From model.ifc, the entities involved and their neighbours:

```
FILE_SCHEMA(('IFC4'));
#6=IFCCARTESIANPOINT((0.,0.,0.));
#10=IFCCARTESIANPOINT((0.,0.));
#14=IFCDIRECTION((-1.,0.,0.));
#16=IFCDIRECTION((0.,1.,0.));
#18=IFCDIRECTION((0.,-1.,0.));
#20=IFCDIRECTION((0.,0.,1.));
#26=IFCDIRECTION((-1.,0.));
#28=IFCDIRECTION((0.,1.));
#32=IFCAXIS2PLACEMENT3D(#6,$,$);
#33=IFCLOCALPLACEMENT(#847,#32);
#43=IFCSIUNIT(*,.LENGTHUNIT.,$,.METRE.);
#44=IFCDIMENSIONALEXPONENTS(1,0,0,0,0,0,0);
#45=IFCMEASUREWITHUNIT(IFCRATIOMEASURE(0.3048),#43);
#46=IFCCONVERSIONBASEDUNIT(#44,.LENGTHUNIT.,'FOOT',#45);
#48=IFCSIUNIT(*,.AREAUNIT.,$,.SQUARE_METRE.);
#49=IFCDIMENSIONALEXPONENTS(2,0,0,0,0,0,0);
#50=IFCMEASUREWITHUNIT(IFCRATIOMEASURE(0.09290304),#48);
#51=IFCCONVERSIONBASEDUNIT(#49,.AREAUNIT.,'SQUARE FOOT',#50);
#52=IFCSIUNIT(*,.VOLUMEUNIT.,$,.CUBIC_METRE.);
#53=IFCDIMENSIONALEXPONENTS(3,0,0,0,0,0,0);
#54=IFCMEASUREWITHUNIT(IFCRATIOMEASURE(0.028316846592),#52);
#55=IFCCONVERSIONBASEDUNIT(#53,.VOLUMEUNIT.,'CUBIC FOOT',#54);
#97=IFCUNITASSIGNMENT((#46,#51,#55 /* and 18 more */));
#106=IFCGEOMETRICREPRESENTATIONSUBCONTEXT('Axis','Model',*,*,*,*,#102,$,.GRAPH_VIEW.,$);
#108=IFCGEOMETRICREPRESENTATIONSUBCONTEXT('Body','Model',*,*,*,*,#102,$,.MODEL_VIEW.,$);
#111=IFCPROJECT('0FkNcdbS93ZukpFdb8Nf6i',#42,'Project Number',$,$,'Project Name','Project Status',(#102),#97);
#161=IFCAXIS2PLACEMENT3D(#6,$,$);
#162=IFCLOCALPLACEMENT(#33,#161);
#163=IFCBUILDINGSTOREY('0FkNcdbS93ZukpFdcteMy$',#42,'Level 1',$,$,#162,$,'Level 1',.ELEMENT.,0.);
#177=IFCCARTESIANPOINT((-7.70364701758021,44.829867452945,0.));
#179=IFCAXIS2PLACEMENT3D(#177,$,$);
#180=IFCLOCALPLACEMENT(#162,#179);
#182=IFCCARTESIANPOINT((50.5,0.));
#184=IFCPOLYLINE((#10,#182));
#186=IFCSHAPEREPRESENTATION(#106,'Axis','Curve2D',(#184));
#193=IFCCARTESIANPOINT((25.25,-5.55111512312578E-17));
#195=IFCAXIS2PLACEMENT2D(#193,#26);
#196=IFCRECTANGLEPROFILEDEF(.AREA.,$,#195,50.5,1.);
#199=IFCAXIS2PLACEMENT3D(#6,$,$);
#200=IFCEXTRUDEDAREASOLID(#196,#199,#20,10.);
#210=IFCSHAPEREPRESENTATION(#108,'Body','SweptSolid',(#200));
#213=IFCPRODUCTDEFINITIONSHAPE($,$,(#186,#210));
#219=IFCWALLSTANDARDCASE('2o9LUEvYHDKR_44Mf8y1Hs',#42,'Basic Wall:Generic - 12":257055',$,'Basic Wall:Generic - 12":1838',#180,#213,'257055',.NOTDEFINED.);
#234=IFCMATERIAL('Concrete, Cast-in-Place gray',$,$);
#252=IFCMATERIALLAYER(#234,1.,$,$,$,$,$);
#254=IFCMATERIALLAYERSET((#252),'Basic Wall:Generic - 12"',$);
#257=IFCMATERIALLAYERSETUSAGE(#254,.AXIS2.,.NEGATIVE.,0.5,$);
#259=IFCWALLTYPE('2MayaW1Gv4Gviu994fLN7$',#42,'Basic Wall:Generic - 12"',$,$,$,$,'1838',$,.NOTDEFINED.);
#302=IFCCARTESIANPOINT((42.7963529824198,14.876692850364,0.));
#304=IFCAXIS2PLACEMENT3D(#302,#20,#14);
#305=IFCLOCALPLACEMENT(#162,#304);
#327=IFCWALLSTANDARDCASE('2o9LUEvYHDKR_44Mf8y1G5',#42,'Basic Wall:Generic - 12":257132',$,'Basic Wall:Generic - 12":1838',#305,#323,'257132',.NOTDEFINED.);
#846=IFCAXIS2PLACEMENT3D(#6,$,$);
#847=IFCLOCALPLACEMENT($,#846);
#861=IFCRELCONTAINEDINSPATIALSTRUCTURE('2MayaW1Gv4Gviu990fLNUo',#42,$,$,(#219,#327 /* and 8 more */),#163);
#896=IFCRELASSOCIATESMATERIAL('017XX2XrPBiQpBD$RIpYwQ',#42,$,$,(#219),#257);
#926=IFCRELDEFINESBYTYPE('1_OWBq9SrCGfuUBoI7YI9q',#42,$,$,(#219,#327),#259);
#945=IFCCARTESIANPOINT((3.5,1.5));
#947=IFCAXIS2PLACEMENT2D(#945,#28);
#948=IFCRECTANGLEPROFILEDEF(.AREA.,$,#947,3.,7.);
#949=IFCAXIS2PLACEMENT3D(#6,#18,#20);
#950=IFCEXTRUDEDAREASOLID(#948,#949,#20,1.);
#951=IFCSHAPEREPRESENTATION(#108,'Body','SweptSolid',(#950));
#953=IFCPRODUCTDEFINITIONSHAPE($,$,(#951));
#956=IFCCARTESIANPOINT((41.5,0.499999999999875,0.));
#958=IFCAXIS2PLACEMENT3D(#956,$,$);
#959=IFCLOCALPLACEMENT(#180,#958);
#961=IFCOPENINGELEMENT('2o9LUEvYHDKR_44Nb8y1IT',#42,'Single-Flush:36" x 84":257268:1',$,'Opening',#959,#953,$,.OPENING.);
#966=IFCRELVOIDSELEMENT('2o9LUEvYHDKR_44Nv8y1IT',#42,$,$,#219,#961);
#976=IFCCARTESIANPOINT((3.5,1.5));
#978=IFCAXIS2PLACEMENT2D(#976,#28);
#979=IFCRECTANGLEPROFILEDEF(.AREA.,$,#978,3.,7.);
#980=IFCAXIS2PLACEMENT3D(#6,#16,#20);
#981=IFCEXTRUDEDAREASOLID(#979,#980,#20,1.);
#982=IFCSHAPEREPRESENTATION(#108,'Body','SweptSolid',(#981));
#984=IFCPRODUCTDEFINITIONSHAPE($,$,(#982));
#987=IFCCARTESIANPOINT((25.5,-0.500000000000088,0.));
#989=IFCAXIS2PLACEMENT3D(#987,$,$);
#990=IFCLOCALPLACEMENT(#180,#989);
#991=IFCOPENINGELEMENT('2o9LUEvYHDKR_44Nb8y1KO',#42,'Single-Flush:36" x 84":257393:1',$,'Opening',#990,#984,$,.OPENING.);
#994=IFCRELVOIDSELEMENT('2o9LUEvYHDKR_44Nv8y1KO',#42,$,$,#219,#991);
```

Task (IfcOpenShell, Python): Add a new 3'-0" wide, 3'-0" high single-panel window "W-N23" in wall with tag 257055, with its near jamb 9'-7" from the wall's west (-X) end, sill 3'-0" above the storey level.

```python
import numpy as np
import ifcopenshell
import ifcopenshell.api.feature
import ifcopenshell.api.geometry
import ifcopenshell.api.root
import ifcopenshell.api.spatial
import ifcopenshell.geom
import ifcopenshell.util.element
import ifcopenshell.util.placement
import ifcopenshell.util.representation
import ifcopenshell.util.shape
import ifcopenshell.util.unit

model = ifcopenshell.open("model.ifc")
unit_scale = ifcopenshell.util.unit.calculate_unit_scale(model)
settings = ifcopenshell.geom.settings()


def volume(element):
    """Net volume in cubic metres, openings subtracted."""
    shape = ifcopenshell.geom.create_shape(settings, element)
    return ifcopenshell.util.shape.get_volume(shape.geometry)


wall = model.by_id(219)
storey = ifcopenshell.util.element.get_container(wall, ifc_class="IfcBuildingStorey")
context = ifcopenshell.util.representation.get_context(model, "Model", "Body", "MODEL_VIEW")
before = volume(wall)

width, height, from_end, sill = 0.9144, 0.9144, 2.921, 0.9144  # metres

# The wall runs along its own X axis, and the end named is its -X end.
wall_shape = ifcopenshell.geom.create_shape(settings, wall)
x, y, z = ifcopenshell.util.shape.get_vertices(wall_shape.geometry).T
start = x.min() + from_end
face, thickness = float(y.min()), float(y.max() - y.min())
wall_matrix = ifcopenshell.util.placement.get_local_placement(wall.ObjectPlacement)
level = ifcopenshell.util.placement.get_local_placement(storey.ObjectPlacement)[2, 3]


def in_wall(x, y):
    """Placement at x, y metres in the wall's axes, at sill height."""
    matrix = wall_matrix.copy()
    matrix[:, 3] = wall_matrix @ np.array([x / unit_scale, y / unit_scale, 0.0, 1.0])
    matrix[2, 3] = level + sill / unit_scale
    return matrix


# Opening: a box that overshoots both wall faces by 50 mm.
opening = ifcopenshell.api.root.create_entity(model, ifc_class="IfcOpeningElement", predefined_type="OPENING")
box = ifcopenshell.api.geometry.add_wall_representation(
    model, context=context, length=width, height=height, thickness=thickness + 0.1
)
ifcopenshell.api.geometry.assign_representation(model, product=opening, representation=box)
ifcopenshell.api.geometry.edit_object_placement(model, product=opening, matrix=in_wall(start, face - 0.05), is_si=False)
ifcopenshell.api.feature.add_feature(model, feature=opening, element=wall)

window = ifcopenshell.api.root.create_entity(model, ifc_class="IfcWindow", name="W-N23", predefined_type="WINDOW")
window.OverallWidth, window.OverallHeight = width / unit_scale, height / unit_scale
window.PartitioningType = "SINGLE_PANEL"
body = ifcopenshell.api.geometry.add_window_representation(
    model,
    context=context,
    overall_width=window.OverallWidth,
    overall_height=window.OverallHeight,
    partition_type="SINGLE_PANEL",
)
ifcopenshell.api.geometry.assign_representation(model, product=window, representation=body)
ifcopenshell.api.spatial.assign_container(model, products=[window], relating_structure=storey)
ifcopenshell.api.feature.add_filling(model, opening=opening, element=window)

# Centre the window in the wall's thickness.
ifcopenshell.api.geometry.edit_object_placement(model, product=window, matrix=in_wall(start, face), is_si=False)
window_shape = ifcopenshell.geom.create_shape(settings, window)
depth = ifcopenshell.util.shape.get_vertices(window_shape.geometry)[:, 1]
offset = face + thickness / 2 - (depth.min() + depth.max()) / 2
ifcopenshell.api.geometry.edit_object_placement(model, product=window, matrix=in_wall(start, offset), is_si=False)

after = volume(wall)

print(f"wall volume {before:.3f} -> {after:.3f} m3")

model.write("model_edited.ifc")
```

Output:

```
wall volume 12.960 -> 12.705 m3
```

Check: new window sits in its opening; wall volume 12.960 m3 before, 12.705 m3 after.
